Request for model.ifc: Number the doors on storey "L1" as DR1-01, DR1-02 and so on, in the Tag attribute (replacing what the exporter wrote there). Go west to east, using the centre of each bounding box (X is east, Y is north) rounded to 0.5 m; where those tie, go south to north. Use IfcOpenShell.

First a look at what the model holds.

```python
import ifcopenshell
import ifcopenshell.util.element
import ifcopenshell.util.placement

model = ifcopenshell.open("model.ifc")
print(model.schema)
storey = next(s for s in model.by_type("IfcBuildingStorey") if s.Name == "L1")
doors = [e for e in ifcopenshell.util.element.get_decomposition(storey) if e.is_a("IfcDoor")]
for e in sorted(doors, key=lambda e: e.id()):
    origin = ifcopenshell.util.placement.get_local_placement(e.ObjectPlacement)[:3, 3]
    print(e.id(), e.Tag, e.Name, origin.round(2) + 0.0, sep=" | ")
```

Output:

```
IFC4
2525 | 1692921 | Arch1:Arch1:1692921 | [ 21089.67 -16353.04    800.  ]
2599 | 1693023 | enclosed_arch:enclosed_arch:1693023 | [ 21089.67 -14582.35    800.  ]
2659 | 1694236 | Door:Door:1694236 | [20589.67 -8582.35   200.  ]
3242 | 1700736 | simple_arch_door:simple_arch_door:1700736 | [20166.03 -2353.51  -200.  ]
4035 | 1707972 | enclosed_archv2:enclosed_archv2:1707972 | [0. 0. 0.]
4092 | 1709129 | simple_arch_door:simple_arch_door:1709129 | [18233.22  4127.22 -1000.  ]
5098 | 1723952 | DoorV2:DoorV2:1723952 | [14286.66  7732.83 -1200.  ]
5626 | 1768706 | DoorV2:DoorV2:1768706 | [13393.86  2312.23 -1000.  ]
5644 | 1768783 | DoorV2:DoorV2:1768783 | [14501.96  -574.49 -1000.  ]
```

```python
import ifcopenshell
import ifcopenshell.geom
import ifcopenshell.util.element
import ifcopenshell.util.shape

model = ifcopenshell.open("model.ifc")
settings = ifcopenshell.geom.settings()
settings.set("use-world-coords", True)


def centre(element):
    shape = ifcopenshell.geom.create_shape(settings, element)
    return ifcopenshell.util.shape.get_bbox_centroid(shape.geometry)


storey = next(s for s in model.by_type("IfcBuildingStorey") if s.Name == "L1")
doors = [e for e in ifcopenshell.util.element.get_decomposition(storey) if e.is_a("IfcDoor")]

# Insertion points can sit at a corner or the storey origin, so sort by the geometry (in metres).
centres = {e: centre(e) for e in doors}
doors.sort(key=lambda e: (round(centres[e][0] / 0.5), centres[e][1]))

for i, e in enumerate(doors, start=1):
    number = f"DR1-{i:02d}"
    e.Tag = number
    print(e.id(), number)

model.write("model_updated.ifc")
```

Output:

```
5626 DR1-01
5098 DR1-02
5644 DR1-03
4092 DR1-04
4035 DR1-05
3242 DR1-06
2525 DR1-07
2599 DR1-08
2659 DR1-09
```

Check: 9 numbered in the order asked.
